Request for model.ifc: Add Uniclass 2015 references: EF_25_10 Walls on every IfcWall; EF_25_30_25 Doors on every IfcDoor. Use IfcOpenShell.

First a look at what the model holds.

```python
import ifcopenshell

model = ifcopenshell.open("model.ifc")
print(model.schema)
print("classifications:", [c.Name for c in model.by_type("IfcClassification")])
for ifc_class in ("IfcDoor", "IfcRoof", "IfcStair", "IfcWall", "IfcWindow"):
    print(ifc_class, len(model.by_type(ifc_class)))
```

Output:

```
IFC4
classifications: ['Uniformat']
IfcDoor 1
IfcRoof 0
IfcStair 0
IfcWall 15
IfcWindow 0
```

```python
import ifcopenshell
import ifcopenshell.api.classification

model = ifcopenshell.open("model.ifc")

system = ifcopenshell.api.classification.add_classification(model, classification="Uniclass 2015")

codes = {
    "IfcWall": ("EF_25_10", "Walls"),
    "IfcDoor": ("EF_25_30_25", "Doors"),
}
for ifc_class, (code, name) in codes.items():
    products = model.by_type(ifc_class)
    ifcopenshell.api.classification.add_reference(
        model, products=products, classification=system, identification=code, name=name
    )
    print(code, len(products))

model.write("model_edited.ifc")
```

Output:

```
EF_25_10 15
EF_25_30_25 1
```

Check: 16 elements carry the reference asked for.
